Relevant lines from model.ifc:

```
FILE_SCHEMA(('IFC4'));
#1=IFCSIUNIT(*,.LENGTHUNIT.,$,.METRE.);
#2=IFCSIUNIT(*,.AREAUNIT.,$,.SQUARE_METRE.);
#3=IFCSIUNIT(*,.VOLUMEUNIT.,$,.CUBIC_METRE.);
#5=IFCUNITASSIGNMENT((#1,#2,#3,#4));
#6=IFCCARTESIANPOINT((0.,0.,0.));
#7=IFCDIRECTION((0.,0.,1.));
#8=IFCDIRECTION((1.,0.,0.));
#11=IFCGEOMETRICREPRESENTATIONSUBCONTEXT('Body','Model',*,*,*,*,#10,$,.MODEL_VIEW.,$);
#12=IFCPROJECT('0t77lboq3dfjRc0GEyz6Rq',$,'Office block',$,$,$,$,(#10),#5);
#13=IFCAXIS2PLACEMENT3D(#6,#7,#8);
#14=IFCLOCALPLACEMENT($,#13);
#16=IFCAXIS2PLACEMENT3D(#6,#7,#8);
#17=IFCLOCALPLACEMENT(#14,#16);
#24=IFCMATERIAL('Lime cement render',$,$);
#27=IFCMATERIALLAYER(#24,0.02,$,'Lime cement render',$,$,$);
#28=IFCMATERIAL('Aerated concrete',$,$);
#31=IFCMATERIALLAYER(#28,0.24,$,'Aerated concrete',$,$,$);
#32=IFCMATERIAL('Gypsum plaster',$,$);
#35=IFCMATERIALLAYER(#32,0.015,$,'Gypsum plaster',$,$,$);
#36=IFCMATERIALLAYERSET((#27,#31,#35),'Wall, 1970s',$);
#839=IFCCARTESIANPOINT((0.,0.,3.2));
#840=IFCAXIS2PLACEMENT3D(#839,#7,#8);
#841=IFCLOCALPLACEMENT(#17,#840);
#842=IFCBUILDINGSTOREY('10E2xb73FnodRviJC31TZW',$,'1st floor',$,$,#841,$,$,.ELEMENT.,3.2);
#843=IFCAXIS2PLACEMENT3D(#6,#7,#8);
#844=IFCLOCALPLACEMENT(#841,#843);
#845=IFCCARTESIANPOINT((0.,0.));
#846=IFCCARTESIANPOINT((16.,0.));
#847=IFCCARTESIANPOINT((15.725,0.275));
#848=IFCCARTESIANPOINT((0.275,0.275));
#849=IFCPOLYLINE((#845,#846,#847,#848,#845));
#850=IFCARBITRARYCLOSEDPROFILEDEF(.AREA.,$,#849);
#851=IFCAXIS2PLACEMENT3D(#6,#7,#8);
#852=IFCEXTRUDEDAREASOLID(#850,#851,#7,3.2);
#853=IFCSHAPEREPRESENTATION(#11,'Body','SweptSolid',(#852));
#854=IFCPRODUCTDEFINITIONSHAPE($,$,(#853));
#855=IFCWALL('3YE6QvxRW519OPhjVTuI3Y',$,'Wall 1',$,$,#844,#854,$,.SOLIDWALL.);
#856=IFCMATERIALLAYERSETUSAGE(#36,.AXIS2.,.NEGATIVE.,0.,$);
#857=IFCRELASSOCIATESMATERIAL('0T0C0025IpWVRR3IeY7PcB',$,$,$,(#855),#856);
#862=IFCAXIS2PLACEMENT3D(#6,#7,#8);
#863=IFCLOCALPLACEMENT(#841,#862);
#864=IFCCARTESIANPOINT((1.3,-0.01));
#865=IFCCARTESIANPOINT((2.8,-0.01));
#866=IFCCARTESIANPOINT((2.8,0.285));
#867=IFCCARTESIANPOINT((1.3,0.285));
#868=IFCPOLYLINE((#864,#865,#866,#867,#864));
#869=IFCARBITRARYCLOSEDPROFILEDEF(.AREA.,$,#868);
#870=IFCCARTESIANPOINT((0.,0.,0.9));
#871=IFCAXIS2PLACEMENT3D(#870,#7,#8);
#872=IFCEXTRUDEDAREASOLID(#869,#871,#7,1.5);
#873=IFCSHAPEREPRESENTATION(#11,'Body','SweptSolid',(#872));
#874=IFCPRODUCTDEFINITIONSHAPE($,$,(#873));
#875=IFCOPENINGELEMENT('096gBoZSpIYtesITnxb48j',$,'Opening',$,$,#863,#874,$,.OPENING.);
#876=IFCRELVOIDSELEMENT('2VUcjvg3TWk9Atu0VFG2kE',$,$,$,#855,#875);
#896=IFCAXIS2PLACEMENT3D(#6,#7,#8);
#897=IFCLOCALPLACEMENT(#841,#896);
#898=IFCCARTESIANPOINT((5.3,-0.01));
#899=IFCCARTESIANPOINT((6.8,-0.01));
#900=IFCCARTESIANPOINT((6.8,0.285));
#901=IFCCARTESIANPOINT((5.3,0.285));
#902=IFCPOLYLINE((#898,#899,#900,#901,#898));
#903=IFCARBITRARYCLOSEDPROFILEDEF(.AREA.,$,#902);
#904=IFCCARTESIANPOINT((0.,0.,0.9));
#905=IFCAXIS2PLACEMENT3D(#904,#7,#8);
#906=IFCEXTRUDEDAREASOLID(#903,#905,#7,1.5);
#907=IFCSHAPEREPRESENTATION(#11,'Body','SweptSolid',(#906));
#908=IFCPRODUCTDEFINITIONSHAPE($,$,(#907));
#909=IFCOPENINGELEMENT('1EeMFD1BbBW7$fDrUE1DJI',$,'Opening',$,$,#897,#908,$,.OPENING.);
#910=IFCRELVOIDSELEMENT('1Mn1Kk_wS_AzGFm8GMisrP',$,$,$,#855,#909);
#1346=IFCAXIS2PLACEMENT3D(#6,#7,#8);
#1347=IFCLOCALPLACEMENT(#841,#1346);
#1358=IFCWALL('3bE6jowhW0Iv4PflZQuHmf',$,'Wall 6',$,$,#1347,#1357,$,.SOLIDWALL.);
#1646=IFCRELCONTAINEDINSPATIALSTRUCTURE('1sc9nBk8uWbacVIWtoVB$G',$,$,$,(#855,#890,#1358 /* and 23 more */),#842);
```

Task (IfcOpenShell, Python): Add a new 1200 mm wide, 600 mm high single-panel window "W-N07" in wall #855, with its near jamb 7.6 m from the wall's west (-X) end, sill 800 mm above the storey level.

```python
import numpy as np
import ifcopenshell
import ifcopenshell.api.feature
import ifcopenshell.api.geometry
import ifcopenshell.api.root
import ifcopenshell.api.spatial
import ifcopenshell.geom
import ifcopenshell.util.element
import ifcopenshell.util.placement
import ifcopenshell.util.representation
import ifcopenshell.util.shape
import ifcopenshell.util.unit

model = ifcopenshell.open("model.ifc")
unit_scale = ifcopenshell.util.unit.calculate_unit_scale(model)
settings = ifcopenshell.geom.settings()


def volume(element):
    """Net volume in cubic metres, openings subtracted."""
    shape = ifcopenshell.geom.create_shape(settings, element)
    return ifcopenshell.util.shape.get_volume(shape.geometry)


wall = model.by_guid("3YE6QvxRW519OPhjVTuI3Y")
storey = ifcopenshell.util.element.get_container(wall, ifc_class="IfcBuildingStorey")
context = ifcopenshell.util.representation.get_context(model, "Model", "Body", "MODEL_VIEW")
before = volume(wall)

width, height, from_end, sill = 1.2, 0.6, 7.6, 0.8  # metres

# The wall runs along its own X axis, and the end named is its -X end.
wall_shape = ifcopenshell.geom.create_shape(settings, wall)
x, y, z = ifcopenshell.util.shape.get_vertices(wall_shape.geometry).T
start = x.min() + from_end
face, thickness = float(y.min()), float(y.max() - y.min())
wall_matrix = ifcopenshell.util.placement.get_local_placement(wall.ObjectPlacement)
level = ifcopenshell.util.placement.get_local_placement(storey.ObjectPlacement)[2, 3]


def in_wall(x, y):
    """Placement at x, y metres in the wall's axes, at sill height."""
    matrix = wall_matrix.copy()
    matrix[:, 3] = wall_matrix @ np.array([x / unit_scale, y / unit_scale, 0.0, 1.0])
    matrix[2, 3] = level + sill / unit_scale
    return matrix


# Opening: a box that overshoots both wall faces by 50 mm.
opening = ifcopenshell.api.root.create_entity(model, ifc_class="IfcOpeningElement", predefined_type="OPENING")
box = ifcopenshell.api.geometry.add_wall_representation(
    model, context=context, length=width, height=height, thickness=thickness + 0.1
)
ifcopenshell.api.geometry.assign_representation(model, product=opening, representation=box)
ifcopenshell.api.geometry.edit_object_placement(model, product=opening, matrix=in_wall(start, face - 0.05), is_si=False)
ifcopenshell.api.feature.add_feature(model, feature=opening, element=wall)

window = ifcopenshell.api.root.create_entity(model, ifc_class="IfcWindow", name="W-N07", predefined_type="WINDOW")
window.OverallWidth, window.OverallHeight = width / unit_scale, height / unit_scale
window.PartitioningType = "SINGLE_PANEL"
body = ifcopenshell.api.geometry.add_window_representation(
    model,
    context=context,
    overall_width=window.OverallWidth,
    overall_height=window.OverallHeight,
    partition_type="SINGLE_PANEL",
)
ifcopenshell.api.geometry.assign_representation(model, product=window, representation=body)
ifcopenshell.api.spatial.assign_container(model, products=[window], relating_structure=storey)
ifcopenshell.api.feature.add_filling(model, opening=opening, element=window)

# Centre the window in the wall's thickness.
ifcopenshell.api.geometry.edit_object_placement(model, product=window, matrix=in_wall(start, face), is_si=False)
window_shape = ifcopenshell.geom.create_shape(settings, window)
depth = ifcopenshell.util.shape.get_vertices(window_shape.geometry)[:, 1]
offset = face + thickness / 2 - (depth.min() + depth.max()) / 2
ifcopenshell.api.geometry.edit_object_placement(model, product=window, matrix=in_wall(start, offset), is_si=False)

after = volume(wall)

print(f"wall volume {before:.3f} -> {after:.3f} m3")

model.write("model_rev.ifc")
```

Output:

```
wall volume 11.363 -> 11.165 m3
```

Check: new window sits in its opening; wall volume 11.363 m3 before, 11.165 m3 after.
